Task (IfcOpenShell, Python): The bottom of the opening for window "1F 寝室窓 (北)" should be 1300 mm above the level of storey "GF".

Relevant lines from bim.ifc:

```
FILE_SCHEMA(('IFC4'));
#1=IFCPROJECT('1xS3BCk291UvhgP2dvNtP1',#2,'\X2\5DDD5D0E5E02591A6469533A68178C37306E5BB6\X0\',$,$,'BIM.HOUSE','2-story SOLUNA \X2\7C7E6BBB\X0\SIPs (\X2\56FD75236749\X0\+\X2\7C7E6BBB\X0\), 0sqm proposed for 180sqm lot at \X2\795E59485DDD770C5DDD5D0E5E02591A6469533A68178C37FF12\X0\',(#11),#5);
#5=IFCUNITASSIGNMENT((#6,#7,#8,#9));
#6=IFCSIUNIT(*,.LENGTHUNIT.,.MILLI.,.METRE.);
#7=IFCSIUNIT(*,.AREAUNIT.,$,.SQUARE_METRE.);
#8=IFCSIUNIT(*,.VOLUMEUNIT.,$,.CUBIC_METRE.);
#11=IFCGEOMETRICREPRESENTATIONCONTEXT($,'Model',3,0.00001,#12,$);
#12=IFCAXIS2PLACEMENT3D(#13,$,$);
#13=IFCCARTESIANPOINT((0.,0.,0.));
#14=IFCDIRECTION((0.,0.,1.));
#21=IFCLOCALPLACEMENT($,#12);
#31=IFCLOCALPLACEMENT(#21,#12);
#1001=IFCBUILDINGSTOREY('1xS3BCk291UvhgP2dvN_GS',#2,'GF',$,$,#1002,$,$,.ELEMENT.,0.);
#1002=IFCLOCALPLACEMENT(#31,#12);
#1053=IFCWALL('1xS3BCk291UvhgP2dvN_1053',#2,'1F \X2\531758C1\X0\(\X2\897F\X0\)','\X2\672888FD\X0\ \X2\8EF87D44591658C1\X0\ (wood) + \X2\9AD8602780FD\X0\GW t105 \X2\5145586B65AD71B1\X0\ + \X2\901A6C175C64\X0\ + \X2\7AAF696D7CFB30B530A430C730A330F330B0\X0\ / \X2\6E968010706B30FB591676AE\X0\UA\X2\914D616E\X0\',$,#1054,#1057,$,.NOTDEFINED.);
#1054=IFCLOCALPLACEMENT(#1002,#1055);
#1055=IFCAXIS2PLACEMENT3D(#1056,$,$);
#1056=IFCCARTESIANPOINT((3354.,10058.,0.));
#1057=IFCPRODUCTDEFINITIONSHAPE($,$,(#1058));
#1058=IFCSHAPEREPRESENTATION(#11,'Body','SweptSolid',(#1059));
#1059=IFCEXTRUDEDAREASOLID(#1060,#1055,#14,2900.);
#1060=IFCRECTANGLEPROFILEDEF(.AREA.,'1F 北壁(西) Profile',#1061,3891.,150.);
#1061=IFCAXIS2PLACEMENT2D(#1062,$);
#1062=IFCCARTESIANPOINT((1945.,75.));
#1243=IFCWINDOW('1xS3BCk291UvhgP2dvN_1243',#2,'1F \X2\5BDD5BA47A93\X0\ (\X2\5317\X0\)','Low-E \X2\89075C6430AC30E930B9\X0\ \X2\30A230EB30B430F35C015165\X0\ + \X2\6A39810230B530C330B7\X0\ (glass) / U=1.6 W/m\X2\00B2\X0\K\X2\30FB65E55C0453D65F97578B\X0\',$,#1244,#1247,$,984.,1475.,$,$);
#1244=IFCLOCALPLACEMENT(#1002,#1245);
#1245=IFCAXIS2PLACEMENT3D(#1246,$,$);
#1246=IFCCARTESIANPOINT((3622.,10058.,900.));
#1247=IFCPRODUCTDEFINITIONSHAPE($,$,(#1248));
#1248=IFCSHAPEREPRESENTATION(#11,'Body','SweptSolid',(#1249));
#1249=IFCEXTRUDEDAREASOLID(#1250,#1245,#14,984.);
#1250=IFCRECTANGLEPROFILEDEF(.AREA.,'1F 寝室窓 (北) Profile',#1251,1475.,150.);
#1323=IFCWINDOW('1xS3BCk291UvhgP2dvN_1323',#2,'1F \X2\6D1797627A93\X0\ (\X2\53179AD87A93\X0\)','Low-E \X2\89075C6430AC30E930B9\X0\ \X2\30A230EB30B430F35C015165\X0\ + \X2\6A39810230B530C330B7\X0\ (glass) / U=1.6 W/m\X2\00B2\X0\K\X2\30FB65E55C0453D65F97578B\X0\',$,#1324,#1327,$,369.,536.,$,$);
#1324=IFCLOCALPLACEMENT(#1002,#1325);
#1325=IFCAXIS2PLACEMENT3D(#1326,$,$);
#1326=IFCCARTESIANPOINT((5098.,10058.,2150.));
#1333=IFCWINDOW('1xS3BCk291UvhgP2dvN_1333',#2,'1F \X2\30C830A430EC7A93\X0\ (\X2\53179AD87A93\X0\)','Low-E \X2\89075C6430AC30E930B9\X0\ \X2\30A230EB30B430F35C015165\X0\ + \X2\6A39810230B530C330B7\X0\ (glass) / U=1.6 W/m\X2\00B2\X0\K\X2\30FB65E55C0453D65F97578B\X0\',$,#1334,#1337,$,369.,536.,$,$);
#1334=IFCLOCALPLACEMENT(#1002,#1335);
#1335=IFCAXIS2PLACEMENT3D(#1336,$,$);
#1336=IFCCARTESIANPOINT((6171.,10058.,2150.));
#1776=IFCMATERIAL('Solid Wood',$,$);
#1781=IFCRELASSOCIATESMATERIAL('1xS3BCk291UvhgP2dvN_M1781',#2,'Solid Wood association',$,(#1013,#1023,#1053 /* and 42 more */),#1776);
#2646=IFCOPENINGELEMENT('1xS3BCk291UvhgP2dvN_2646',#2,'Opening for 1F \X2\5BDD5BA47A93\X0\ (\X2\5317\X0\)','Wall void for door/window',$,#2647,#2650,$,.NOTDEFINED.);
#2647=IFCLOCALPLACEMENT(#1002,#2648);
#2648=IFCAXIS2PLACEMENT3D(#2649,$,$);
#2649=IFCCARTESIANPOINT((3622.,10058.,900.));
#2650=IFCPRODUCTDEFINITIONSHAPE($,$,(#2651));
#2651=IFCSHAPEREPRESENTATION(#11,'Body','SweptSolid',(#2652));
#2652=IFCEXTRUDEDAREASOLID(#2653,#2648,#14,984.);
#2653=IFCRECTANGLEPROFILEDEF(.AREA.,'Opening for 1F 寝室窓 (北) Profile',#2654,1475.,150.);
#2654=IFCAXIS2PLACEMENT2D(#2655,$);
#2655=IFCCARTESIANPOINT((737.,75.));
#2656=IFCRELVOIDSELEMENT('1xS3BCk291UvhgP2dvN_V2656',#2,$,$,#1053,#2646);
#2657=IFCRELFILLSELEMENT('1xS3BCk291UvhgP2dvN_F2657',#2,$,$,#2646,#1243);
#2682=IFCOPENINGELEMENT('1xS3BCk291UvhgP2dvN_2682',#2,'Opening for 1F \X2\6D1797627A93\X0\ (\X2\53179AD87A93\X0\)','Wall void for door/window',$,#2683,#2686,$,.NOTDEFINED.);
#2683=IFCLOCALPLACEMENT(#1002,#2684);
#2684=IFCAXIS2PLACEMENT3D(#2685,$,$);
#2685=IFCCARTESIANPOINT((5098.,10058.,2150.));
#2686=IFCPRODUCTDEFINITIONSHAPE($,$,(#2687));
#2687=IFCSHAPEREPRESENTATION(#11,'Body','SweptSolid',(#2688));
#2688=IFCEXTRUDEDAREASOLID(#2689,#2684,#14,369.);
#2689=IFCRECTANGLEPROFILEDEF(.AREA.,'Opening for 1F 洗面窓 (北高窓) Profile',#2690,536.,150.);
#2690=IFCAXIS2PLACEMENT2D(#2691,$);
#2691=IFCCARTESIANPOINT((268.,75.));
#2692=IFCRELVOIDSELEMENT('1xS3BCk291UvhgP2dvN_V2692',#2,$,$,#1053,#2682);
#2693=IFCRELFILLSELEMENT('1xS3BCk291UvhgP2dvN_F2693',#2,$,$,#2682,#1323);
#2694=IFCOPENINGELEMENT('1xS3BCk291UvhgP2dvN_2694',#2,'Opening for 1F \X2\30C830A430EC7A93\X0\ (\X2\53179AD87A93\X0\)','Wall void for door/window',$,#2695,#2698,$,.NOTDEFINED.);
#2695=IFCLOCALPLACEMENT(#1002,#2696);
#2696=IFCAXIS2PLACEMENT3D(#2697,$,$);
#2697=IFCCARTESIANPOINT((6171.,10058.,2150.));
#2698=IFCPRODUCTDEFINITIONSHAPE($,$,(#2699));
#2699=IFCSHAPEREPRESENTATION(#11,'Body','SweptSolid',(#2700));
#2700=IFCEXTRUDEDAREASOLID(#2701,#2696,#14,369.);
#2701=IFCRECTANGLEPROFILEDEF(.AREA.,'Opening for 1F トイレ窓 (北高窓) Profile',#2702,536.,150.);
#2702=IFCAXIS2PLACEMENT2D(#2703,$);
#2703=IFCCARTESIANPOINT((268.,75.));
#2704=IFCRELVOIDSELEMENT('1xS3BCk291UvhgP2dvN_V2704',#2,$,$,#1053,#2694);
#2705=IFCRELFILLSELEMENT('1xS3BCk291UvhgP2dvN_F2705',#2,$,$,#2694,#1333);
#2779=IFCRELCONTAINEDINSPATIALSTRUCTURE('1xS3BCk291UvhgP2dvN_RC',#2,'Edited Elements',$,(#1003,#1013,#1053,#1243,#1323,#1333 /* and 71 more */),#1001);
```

```python
import numpy as np
import ifcopenshell
import ifcopenshell.api.geometry
import ifcopenshell.geom
import ifcopenshell.util.element
import ifcopenshell.util.placement
import ifcopenshell.util.shape
import ifcopenshell.util.unit

model = ifcopenshell.open("bim.ifc")
unit_scale = ifcopenshell.util.unit.calculate_unit_scale(model)

window = model.by_id(1243)
opening = window.FillsVoids[0].RelatingOpeningElement
storey = ifcopenshell.util.element.get_container(window, ifc_class="IfcBuildingStorey")
level = ifcopenshell.util.placement.get_local_placement(storey.ObjectPlacement)[2, 3]

# The opening's origin need not be at the sill, so measure its lowest point.
shape = ifcopenshell.geom.create_shape(ifcopenshell.geom.settings(), opening)
bottom = ifcopenshell.util.shape.get_shape_bottom_elevation(shape, shape.geometry) / unit_scale
dz = level + 1300.0 - bottom

shift = np.array([0.0, 0.0, dz])
# The window is not placed relative to its opening, so move both.
for product in (opening, window):
    matrix = ifcopenshell.util.placement.get_local_placement(product.ObjectPlacement)
    matrix[:3, 3] += shift
    ifcopenshell.api.geometry.edit_object_placement(model, product=product, matrix=matrix, is_si=False)

print(f"moved by {dz * unit_scale:+.3f} m")

model.write("bim-out.ifc")
```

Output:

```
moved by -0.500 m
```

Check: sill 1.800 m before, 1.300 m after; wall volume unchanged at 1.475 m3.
